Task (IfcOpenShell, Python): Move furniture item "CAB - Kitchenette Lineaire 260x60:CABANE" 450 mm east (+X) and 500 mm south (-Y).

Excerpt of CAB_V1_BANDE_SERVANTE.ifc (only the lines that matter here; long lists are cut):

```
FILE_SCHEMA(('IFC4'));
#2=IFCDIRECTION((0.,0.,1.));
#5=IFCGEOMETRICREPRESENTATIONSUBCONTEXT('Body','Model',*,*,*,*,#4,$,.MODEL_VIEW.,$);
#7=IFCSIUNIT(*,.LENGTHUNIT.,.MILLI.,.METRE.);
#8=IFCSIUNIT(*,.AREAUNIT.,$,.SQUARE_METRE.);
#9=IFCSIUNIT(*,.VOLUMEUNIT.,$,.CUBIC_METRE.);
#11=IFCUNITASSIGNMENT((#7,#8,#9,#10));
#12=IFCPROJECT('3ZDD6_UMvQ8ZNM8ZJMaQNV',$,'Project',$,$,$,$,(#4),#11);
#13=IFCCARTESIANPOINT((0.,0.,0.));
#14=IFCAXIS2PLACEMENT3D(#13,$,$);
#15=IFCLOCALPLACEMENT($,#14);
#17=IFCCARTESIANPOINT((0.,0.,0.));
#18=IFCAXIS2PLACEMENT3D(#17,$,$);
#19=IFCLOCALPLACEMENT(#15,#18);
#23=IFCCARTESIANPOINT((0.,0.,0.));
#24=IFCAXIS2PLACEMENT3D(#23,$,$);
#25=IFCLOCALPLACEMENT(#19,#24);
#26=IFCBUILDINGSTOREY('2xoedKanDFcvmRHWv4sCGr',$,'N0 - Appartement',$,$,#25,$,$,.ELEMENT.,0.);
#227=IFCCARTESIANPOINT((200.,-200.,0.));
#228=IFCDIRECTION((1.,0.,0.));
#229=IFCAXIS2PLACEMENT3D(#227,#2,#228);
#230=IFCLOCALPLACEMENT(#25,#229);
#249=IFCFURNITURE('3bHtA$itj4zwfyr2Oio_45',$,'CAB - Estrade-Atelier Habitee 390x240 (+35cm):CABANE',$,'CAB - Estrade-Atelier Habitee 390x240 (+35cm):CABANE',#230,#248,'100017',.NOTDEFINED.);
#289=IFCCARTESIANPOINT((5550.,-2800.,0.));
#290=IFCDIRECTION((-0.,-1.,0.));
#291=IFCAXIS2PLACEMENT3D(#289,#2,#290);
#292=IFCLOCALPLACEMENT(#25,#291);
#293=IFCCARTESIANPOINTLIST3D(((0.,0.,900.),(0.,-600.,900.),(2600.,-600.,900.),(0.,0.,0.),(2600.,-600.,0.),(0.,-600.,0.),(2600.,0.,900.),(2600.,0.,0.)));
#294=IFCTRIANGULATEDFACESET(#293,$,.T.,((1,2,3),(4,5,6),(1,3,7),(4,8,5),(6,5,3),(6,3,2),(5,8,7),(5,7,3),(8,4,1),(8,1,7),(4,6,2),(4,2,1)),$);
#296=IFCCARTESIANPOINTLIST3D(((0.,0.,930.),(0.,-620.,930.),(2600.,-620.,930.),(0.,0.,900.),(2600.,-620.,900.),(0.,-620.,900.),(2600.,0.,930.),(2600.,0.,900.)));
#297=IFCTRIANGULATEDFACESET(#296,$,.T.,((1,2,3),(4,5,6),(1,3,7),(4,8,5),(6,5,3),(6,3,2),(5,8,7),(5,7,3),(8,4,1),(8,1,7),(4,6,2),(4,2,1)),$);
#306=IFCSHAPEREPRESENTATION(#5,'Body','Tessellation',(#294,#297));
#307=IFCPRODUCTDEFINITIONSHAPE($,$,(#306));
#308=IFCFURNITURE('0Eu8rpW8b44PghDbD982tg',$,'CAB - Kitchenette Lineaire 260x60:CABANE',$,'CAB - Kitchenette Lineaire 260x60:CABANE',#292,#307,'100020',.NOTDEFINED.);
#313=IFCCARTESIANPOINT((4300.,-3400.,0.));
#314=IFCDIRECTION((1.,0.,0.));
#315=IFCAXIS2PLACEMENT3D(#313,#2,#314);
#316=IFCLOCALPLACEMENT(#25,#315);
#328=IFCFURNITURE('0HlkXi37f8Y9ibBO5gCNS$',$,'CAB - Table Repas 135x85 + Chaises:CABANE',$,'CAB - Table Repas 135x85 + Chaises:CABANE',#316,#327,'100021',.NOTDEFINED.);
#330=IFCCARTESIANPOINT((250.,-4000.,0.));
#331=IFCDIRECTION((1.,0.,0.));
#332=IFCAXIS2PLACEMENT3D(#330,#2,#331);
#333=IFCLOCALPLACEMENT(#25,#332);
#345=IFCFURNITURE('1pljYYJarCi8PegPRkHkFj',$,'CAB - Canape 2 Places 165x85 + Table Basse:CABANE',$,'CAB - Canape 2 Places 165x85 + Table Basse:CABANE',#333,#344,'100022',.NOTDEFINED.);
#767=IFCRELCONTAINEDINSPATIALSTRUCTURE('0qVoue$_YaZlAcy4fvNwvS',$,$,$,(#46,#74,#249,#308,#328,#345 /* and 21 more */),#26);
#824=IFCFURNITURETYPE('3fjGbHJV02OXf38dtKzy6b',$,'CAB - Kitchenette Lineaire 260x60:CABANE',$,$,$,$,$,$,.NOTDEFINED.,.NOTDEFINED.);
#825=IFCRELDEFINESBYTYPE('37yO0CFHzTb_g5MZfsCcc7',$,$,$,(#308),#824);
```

```python
import ifcopenshell
import ifcopenshell.api.geometry
import ifcopenshell.util.placement

model = ifcopenshell.open("CAB_V1_BANDE_SERVANTE.ifc")

item = model.by_guid("0Eu8rpW8b44PghDbD982tg")
matrix = ifcopenshell.util.placement.get_local_placement(item.ObjectPlacement)
matrix[0, 3] += 450.0
matrix[1, 3] -= 500.0
ifcopenshell.api.geometry.edit_object_placement(model, product=item, matrix=matrix, is_si=False)

print(ifcopenshell.util.placement.get_local_placement(item.ObjectPlacement).round(3) + 0.0)

model.write("CAB_V1_BANDE_SERVANTE_edited.ifc")
```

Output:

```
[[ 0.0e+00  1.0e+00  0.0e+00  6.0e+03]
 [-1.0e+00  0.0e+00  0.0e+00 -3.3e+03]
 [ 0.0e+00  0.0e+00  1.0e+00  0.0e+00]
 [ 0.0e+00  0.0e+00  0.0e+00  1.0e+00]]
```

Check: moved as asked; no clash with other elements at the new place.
